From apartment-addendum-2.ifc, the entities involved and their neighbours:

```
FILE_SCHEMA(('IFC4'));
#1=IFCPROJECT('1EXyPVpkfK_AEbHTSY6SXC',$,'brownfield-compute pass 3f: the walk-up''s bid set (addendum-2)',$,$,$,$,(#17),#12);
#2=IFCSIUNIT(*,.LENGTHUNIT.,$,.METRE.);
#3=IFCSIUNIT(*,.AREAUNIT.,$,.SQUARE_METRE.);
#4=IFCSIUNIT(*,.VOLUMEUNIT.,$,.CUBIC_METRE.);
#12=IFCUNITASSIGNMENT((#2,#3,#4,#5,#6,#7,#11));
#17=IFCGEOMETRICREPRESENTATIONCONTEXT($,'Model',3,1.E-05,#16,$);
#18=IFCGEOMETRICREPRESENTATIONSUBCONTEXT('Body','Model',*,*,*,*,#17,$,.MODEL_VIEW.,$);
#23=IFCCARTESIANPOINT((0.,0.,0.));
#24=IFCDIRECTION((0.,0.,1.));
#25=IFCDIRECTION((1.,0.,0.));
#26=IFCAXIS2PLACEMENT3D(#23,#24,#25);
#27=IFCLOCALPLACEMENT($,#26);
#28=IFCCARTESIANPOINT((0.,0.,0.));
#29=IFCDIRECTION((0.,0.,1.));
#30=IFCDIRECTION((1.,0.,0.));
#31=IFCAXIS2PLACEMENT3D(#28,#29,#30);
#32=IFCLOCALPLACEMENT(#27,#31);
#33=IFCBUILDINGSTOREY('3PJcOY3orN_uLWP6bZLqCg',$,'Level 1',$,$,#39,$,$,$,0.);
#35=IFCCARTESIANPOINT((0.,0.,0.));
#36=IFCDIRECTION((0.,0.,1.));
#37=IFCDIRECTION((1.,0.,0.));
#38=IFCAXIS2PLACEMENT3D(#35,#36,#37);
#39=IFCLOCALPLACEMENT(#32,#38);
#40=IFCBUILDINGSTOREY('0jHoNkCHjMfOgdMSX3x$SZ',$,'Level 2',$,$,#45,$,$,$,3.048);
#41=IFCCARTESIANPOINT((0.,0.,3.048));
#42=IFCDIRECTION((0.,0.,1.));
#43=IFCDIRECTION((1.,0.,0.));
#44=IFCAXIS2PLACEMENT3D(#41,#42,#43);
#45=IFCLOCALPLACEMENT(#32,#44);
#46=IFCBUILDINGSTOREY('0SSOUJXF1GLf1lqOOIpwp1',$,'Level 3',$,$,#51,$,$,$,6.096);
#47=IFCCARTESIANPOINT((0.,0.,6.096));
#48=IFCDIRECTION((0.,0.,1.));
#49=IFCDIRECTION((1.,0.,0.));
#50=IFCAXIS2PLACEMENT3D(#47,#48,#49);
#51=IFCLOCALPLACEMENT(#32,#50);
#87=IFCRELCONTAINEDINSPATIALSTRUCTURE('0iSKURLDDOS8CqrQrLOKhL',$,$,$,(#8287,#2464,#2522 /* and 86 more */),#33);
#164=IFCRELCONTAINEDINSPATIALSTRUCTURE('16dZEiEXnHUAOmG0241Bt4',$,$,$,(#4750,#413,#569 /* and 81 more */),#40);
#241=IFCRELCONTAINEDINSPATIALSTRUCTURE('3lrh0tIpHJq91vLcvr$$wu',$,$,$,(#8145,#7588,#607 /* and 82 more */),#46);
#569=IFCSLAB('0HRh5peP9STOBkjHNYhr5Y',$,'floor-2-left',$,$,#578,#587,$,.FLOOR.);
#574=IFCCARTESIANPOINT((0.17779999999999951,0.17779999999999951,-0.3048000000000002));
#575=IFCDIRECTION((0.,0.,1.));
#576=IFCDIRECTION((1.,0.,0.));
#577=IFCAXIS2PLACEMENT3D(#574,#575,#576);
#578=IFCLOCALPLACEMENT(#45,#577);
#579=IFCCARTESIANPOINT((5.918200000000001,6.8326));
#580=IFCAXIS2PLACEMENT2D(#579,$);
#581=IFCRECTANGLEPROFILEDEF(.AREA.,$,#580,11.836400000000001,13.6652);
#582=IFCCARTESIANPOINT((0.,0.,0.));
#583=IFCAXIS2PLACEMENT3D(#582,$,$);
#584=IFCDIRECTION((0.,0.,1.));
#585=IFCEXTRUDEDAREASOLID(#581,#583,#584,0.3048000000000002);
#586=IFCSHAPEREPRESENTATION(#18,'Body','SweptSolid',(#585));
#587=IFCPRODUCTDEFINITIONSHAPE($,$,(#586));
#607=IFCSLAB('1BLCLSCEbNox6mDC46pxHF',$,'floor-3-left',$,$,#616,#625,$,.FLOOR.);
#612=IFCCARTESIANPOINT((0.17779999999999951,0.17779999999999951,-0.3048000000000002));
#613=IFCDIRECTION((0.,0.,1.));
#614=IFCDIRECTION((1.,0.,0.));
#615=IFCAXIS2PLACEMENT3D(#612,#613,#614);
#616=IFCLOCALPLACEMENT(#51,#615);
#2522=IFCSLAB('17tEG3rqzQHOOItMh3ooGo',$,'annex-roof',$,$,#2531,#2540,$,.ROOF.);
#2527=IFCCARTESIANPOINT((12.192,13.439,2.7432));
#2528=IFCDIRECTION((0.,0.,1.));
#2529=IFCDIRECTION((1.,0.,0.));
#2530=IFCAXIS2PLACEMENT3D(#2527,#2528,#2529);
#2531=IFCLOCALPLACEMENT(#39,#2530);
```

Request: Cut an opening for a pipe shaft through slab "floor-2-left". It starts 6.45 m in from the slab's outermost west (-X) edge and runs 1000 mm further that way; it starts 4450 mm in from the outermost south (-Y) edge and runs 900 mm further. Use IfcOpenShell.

```python
import numpy as np
import ifcopenshell
import ifcopenshell.api.feature
import ifcopenshell.api.geometry
import ifcopenshell.api.root
import ifcopenshell.geom
import ifcopenshell.util.placement
import ifcopenshell.util.representation
import ifcopenshell.util.shape
import ifcopenshell.util.unit

model = ifcopenshell.open("apartment-addendum-2.ifc")
unit_scale = ifcopenshell.util.unit.calculate_unit_scale(model)
settings = ifcopenshell.geom.settings()


def volume(element):
    """Net volume in cubic metres, openings subtracted."""
    shape = ifcopenshell.geom.create_shape(settings, element)
    return ifcopenshell.util.shape.get_volume(shape.geometry)


slab = model.by_id(569)
before = volume(slab)

# Extent in the slab's own axes, in metres. The edges named are its -X and -Y sides.
slab_shape = ifcopenshell.geom.create_shape(settings, slab)
vertices = ifcopenshell.util.shape.get_vertices(slab_shape.geometry)
x_min, y_min, bottom = vertices.min(axis=0)
top = vertices[:, 2].max()

opening = ifcopenshell.api.root.create_entity(model, ifc_class="IfcOpeningElement", name="Pipe shaft opening", predefined_type="OPENING")
context = ifcopenshell.util.representation.get_context(model, "Model", "Body", "MODEL_VIEW")
width, depth = 1, 0.9
outline = [(0.0, 0.0), (width, 0.0), (width, depth), (0.0, depth), (0.0, 0.0)]
# Overshoot both faces by 50 mm so the cut is clean.
shape = ifcopenshell.api.geometry.add_slab_representation(
    model, context=context, depth=top - bottom + 0.1, polyline=outline
)
ifcopenshell.api.geometry.assign_representation(model, product=opening, representation=shape)

matrix = ifcopenshell.util.placement.get_local_placement(slab.ObjectPlacement)
matrix[:, 3] = matrix @ np.append(np.array([x_min + 6.45, y_min + 4.45, bottom - 0.05]) / unit_scale, 1.0)
ifcopenshell.api.geometry.edit_object_placement(model, product=opening, matrix=matrix, is_si=False)
ifcopenshell.api.feature.add_feature(model, feature=opening, element=slab)

after = volume(slab)

print(f"slab volume {before:.3f} -> {after:.3f} m3")

model.write("apartment-addendum-2_edited.ifc")
```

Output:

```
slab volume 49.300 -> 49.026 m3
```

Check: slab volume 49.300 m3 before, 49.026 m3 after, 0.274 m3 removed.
